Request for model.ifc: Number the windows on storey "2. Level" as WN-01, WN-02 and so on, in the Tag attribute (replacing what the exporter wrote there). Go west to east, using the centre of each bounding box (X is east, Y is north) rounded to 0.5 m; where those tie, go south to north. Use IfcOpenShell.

First a look at what the model holds.

```python
import ifcopenshell
import ifcopenshell.util.element
import ifcopenshell.util.placement

model = ifcopenshell.open("model.ifc")
print(model.schema)
storey = next(s for s in model.by_type("IfcBuildingStorey") if s.Name == "2. Level")
windows = [e for e in ifcopenshell.util.element.get_decomposition(storey) if e.is_a("IfcWindow")]
for e in sorted(windows, key=lambda e: e.id()):
    origin = ifcopenshell.util.placement.get_local_placement(e.ObjectPlacement)[:3, 3]
    print(e.id(), e.Tag, e.Name, origin.round(2) + 0.0, sep=" | ")
```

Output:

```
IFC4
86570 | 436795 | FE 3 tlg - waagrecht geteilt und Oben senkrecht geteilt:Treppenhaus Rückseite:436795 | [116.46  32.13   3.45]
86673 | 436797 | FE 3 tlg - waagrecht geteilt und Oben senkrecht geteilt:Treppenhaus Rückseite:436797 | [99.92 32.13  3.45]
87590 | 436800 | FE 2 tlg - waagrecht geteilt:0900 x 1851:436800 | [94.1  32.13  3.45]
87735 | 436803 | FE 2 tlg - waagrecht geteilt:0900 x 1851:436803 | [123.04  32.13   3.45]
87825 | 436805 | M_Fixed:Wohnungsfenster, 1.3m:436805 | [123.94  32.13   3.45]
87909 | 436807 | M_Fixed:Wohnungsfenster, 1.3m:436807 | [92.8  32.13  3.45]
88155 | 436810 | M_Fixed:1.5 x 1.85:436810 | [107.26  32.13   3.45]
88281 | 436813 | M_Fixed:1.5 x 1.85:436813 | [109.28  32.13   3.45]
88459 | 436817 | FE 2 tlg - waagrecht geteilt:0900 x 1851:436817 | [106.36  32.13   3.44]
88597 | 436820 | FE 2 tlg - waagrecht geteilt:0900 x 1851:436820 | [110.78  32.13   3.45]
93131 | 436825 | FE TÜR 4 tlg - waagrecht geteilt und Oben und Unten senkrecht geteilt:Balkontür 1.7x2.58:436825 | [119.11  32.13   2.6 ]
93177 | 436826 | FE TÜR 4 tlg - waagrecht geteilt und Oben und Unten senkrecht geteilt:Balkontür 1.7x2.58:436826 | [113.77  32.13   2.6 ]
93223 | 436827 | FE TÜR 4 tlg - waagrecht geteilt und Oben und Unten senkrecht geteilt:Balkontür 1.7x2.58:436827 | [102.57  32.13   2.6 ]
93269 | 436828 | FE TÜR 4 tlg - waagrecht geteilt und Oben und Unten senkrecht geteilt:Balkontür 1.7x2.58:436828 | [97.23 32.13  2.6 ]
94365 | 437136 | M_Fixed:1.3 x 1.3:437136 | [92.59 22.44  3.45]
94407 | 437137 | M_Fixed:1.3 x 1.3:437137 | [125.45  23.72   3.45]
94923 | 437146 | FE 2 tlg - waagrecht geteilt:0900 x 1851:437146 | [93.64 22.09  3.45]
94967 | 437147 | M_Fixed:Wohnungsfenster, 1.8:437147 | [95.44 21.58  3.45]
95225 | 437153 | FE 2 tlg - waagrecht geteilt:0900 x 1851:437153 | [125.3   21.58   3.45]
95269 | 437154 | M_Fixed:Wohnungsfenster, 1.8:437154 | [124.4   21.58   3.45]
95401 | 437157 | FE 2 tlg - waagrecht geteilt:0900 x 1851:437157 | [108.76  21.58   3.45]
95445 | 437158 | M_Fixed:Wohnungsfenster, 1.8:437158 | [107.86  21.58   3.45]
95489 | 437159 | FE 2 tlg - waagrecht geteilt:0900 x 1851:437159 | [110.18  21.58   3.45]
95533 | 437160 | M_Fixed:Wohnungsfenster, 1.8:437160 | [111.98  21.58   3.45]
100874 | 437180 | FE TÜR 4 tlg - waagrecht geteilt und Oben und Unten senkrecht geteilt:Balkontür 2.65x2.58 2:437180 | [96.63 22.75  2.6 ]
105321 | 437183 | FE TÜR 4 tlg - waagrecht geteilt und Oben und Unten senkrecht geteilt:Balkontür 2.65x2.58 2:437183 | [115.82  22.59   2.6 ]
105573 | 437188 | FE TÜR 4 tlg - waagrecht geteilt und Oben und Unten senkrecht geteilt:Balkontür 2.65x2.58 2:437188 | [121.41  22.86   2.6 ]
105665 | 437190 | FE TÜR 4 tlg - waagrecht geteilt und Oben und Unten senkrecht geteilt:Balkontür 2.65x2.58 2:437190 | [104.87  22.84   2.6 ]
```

```python
import ifcopenshell
import ifcopenshell.geom
import ifcopenshell.util.element
import ifcopenshell.util.shape

model = ifcopenshell.open("model.ifc")
settings = ifcopenshell.geom.settings()
settings.set("use-world-coords", True)


def centre(element):
    shape = ifcopenshell.geom.create_shape(settings, element)
    return ifcopenshell.util.shape.get_bbox_centroid(shape.geometry)


storey = next(s for s in model.by_type("IfcBuildingStorey") if s.Name == "2. Level")
windows = [e for e in ifcopenshell.util.element.get_decomposition(storey) if e.is_a("IfcWindow")]

# Insertion points can sit at a corner or the storey origin, so sort by the geometry (in metres).
centres = {e: centre(e) for e in windows}
windows.sort(key=lambda e: (round(centres[e][0] / 0.5), centres[e][1]))

for i, e in enumerate(windows, start=1):
    number = f"WN-{i:02d}"
    e.Tag = number
    print(e.id(), number)

model.write("model-out.ifc")
```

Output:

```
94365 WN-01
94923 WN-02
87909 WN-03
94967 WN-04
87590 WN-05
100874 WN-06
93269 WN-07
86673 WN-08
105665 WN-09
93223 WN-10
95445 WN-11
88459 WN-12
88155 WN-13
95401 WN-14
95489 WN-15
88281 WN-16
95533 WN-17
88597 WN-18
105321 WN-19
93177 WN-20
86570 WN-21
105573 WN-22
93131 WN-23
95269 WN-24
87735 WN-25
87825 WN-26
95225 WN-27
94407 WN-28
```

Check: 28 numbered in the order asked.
